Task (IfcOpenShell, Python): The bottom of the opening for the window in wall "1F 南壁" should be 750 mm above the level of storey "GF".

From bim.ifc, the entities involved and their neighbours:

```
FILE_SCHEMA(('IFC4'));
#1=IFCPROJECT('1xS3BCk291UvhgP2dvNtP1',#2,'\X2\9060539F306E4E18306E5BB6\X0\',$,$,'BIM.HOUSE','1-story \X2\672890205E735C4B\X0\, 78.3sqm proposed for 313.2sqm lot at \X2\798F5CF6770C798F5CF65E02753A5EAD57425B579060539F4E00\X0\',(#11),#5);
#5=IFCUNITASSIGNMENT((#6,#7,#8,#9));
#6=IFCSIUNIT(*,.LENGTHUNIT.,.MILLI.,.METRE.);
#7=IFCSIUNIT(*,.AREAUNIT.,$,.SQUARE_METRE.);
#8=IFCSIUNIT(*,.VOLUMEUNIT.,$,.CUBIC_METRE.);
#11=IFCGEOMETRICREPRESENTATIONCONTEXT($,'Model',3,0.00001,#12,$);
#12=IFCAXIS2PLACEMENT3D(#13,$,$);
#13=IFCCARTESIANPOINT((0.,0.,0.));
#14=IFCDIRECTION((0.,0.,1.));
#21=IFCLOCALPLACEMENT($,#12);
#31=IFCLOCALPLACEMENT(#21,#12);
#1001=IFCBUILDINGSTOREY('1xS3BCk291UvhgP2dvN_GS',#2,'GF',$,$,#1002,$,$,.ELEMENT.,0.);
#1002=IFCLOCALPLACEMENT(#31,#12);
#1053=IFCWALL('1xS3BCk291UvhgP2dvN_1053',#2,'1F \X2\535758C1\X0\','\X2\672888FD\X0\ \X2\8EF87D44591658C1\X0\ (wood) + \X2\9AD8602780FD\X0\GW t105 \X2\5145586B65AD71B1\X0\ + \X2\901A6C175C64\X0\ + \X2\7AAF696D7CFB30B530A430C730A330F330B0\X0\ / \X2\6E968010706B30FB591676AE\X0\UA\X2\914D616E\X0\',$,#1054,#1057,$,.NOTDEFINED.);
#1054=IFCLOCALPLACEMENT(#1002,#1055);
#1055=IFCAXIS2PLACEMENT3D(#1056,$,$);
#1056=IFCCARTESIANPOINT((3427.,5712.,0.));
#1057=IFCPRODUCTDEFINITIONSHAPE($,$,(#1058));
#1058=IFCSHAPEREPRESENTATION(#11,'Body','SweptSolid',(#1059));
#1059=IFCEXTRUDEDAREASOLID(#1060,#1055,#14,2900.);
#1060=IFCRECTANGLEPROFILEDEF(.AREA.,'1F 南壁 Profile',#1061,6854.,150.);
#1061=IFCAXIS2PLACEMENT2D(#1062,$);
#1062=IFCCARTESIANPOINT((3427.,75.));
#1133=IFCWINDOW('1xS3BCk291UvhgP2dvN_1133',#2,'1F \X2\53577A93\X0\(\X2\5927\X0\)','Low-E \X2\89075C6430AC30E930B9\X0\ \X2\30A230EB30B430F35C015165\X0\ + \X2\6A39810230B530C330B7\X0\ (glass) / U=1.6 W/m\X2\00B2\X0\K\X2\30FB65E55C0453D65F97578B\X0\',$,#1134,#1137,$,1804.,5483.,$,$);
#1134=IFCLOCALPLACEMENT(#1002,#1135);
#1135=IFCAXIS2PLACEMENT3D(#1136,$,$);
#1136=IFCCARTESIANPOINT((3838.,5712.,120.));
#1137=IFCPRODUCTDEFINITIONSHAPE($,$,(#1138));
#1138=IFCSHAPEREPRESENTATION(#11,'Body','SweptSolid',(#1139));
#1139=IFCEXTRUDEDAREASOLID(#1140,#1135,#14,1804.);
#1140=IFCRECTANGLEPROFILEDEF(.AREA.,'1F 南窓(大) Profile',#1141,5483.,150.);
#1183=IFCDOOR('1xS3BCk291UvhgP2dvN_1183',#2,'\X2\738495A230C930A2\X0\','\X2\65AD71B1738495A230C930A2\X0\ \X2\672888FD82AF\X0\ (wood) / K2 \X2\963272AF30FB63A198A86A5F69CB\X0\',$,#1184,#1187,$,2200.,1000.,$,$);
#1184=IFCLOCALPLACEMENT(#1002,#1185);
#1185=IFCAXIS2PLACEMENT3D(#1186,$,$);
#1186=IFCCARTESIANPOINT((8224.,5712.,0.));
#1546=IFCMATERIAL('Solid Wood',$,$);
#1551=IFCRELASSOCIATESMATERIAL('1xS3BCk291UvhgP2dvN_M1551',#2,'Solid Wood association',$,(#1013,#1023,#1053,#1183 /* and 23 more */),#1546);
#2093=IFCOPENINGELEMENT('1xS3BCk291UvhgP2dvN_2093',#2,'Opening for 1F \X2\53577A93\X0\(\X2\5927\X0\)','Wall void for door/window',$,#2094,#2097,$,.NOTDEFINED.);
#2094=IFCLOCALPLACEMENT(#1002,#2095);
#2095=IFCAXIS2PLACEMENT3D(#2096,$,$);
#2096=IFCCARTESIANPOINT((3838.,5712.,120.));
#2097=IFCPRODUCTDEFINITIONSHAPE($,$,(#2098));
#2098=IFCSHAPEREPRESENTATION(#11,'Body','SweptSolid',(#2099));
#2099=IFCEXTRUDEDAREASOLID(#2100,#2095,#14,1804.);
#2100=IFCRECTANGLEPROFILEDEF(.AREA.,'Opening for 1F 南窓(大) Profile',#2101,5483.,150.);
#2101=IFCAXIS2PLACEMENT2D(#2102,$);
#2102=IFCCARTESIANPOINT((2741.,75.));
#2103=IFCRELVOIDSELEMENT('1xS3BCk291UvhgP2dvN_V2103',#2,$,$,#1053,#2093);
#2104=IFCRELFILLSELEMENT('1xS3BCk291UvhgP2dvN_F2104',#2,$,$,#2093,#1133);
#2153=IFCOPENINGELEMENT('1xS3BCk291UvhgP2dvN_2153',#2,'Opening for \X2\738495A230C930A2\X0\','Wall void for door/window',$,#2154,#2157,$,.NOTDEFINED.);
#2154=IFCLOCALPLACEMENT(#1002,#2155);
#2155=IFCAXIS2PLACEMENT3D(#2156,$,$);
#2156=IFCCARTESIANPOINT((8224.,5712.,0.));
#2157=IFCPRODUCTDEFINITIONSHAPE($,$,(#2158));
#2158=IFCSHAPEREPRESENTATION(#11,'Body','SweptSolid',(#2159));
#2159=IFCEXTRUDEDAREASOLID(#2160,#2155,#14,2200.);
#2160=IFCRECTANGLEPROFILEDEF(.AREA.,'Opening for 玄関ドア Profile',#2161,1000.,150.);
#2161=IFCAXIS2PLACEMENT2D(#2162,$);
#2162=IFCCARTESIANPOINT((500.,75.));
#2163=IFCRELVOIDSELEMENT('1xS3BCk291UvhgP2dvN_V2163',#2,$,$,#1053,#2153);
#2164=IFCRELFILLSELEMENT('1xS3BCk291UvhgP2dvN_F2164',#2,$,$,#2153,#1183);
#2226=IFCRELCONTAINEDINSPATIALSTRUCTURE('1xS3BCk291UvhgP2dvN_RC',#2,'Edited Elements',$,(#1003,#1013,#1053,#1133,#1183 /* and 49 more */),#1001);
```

```python
import numpy as np
import ifcopenshell
import ifcopenshell.api.geometry
import ifcopenshell.geom
import ifcopenshell.util.element
import ifcopenshell.util.placement
import ifcopenshell.util.shape
import ifcopenshell.util.unit

model = ifcopenshell.open("bim.ifc")
unit_scale = ifcopenshell.util.unit.calculate_unit_scale(model)

window = model.by_guid("1xS3BCk291UvhgP2dvN_1133")
opening = window.FillsVoids[0].RelatingOpeningElement
storey = ifcopenshell.util.element.get_container(window, ifc_class="IfcBuildingStorey")
level = ifcopenshell.util.placement.get_local_placement(storey.ObjectPlacement)[2, 3]

# The opening's origin need not be at the sill, so measure its lowest point.
shape = ifcopenshell.geom.create_shape(ifcopenshell.geom.settings(), opening)
bottom = ifcopenshell.util.shape.get_shape_bottom_elevation(shape, shape.geometry) / unit_scale
dz = level + 0.75 / unit_scale - bottom

shift = np.array([0.0, 0.0, dz])
# The window is not placed relative to its opening, so move both.
for product in (opening, window):
    matrix = ifcopenshell.util.placement.get_local_placement(product.ObjectPlacement)
    matrix[:3, 3] += shift
    ifcopenshell.api.geometry.edit_object_placement(model, product=product, matrix=matrix, is_si=False)

print(f"moved by {dz * unit_scale:+.3f} m")

model.write("bim_rev.ifc")
```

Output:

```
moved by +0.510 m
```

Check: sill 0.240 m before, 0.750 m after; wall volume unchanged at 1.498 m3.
